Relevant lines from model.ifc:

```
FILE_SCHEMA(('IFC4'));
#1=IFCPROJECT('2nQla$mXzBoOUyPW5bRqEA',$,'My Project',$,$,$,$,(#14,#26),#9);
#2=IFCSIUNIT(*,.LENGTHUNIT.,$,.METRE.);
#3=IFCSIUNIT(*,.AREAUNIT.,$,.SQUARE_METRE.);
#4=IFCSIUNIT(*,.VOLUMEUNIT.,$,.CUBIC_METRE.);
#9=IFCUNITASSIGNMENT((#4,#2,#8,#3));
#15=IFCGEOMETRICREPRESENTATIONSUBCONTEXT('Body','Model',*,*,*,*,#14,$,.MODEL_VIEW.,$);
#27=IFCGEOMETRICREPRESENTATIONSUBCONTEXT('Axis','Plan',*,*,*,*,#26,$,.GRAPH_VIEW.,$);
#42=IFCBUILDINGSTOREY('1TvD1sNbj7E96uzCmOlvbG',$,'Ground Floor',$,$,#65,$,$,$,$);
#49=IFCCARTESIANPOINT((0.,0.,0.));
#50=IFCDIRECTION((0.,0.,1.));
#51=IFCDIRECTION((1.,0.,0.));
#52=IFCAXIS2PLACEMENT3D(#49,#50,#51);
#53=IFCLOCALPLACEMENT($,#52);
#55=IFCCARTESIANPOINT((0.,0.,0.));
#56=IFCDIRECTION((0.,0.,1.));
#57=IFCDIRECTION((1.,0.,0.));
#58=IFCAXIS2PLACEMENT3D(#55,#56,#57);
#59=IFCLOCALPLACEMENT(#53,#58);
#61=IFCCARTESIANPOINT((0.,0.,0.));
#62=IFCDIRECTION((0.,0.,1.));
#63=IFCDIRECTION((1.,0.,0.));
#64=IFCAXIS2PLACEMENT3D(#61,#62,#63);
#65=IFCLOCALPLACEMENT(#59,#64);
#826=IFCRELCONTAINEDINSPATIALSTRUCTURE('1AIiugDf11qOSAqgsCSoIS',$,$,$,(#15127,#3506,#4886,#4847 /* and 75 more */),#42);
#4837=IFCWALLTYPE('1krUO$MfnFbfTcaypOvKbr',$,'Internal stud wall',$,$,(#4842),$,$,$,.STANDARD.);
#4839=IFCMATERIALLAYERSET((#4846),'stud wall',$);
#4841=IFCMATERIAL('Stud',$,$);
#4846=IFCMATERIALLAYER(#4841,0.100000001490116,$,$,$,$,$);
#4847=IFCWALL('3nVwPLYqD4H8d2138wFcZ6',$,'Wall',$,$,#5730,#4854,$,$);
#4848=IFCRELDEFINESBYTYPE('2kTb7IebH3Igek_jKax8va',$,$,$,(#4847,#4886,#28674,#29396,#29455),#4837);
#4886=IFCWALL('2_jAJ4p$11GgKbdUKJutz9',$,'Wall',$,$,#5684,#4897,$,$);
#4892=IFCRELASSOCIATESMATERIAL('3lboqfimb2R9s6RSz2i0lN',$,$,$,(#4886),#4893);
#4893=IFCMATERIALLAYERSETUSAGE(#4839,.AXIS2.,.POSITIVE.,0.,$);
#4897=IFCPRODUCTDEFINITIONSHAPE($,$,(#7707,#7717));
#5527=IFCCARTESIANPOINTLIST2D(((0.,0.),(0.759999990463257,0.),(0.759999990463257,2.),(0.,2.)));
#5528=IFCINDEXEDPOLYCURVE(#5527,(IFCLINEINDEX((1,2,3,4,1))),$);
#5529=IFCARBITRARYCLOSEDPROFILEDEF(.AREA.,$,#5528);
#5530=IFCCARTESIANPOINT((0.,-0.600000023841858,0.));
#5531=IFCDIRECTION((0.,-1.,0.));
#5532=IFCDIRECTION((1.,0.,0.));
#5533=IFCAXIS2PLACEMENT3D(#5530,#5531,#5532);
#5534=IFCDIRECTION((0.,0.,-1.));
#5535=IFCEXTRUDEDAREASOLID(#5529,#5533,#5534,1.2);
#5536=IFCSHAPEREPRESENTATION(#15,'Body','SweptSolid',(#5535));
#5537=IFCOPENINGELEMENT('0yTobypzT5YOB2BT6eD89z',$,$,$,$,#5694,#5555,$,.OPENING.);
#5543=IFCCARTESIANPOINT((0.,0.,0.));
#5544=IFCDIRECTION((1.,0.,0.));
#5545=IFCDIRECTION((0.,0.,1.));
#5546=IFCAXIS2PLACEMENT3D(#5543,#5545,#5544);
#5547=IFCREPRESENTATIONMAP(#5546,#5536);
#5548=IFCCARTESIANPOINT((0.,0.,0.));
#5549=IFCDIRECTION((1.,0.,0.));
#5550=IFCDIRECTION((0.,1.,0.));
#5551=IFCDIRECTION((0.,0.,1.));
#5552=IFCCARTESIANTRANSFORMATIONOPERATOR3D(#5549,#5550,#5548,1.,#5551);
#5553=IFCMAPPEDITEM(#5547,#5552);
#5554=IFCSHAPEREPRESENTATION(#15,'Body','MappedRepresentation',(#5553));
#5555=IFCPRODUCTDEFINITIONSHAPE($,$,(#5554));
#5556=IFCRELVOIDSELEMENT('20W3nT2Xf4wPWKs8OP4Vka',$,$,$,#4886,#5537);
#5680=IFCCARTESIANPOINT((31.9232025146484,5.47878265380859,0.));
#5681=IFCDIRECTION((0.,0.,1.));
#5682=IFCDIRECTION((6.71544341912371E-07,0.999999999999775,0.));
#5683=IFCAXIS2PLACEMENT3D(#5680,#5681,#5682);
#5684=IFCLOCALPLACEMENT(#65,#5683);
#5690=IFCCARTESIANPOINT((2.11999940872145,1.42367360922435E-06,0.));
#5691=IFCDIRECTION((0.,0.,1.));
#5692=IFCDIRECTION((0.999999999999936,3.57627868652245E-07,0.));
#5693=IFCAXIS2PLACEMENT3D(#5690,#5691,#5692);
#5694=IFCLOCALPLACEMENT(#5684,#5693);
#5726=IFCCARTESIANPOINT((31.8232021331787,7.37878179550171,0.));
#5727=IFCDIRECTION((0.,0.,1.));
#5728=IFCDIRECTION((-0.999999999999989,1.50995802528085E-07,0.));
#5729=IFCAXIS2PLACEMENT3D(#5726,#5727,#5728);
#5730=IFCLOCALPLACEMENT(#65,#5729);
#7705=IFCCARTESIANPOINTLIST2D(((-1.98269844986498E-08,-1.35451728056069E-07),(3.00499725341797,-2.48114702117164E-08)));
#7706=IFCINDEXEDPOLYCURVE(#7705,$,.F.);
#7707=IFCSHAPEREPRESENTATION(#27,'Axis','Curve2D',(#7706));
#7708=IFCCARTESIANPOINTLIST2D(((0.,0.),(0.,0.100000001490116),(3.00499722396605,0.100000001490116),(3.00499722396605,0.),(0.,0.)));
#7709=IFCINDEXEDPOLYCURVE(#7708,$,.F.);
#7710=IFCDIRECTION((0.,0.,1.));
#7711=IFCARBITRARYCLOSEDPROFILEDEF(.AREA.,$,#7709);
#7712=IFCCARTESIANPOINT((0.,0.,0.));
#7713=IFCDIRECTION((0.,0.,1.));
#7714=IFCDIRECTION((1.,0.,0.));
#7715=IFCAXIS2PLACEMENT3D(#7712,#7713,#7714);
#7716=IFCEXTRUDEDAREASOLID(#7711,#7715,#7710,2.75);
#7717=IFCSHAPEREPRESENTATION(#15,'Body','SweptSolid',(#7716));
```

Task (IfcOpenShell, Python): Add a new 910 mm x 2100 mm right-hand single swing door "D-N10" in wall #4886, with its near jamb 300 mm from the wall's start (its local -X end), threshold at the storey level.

```python
import numpy as np
import ifcopenshell
import ifcopenshell.api.feature
import ifcopenshell.api.geometry
import ifcopenshell.api.root
import ifcopenshell.api.spatial
import ifcopenshell.geom
import ifcopenshell.util.element
import ifcopenshell.util.placement
import ifcopenshell.util.representation
import ifcopenshell.util.shape
import ifcopenshell.util.unit

model = ifcopenshell.open("model.ifc")
unit_scale = ifcopenshell.util.unit.calculate_unit_scale(model)
settings = ifcopenshell.geom.settings()


def volume(element):
    """Net volume in cubic metres, openings subtracted."""
    shape = ifcopenshell.geom.create_shape(settings, element)
    return ifcopenshell.util.shape.get_volume(shape.geometry)


wall = model.by_id(4886)
storey = ifcopenshell.util.element.get_container(wall, ifc_class="IfcBuildingStorey")
context = ifcopenshell.util.representation.get_context(model, "Model", "Body", "MODEL_VIEW")
before = volume(wall)

width, height, from_end, sill = 0.91, 2.1, 0.3, 0.0  # metres

# The wall runs along its own X axis, and the end named is its -X end.
wall_shape = ifcopenshell.geom.create_shape(settings, wall)
x, y, z = ifcopenshell.util.shape.get_vertices(wall_shape.geometry).T
start = x.min() + from_end
face, thickness = float(y.min()), float(y.max() - y.min())
wall_matrix = ifcopenshell.util.placement.get_local_placement(wall.ObjectPlacement)
level = ifcopenshell.util.placement.get_local_placement(storey.ObjectPlacement)[2, 3]


def in_wall(x, y):
    """Placement at x, y metres in the wall's axes, at sill height."""
    matrix = wall_matrix.copy()
    matrix[:, 3] = wall_matrix @ np.array([x / unit_scale, y / unit_scale, 0.0, 1.0])
    matrix[2, 3] = level + sill / unit_scale
    return matrix


# Opening: a box that overshoots both wall faces by 50 mm.
opening = ifcopenshell.api.root.create_entity(model, ifc_class="IfcOpeningElement", predefined_type="OPENING")
box = ifcopenshell.api.geometry.add_wall_representation(
    model, context=context, length=width, height=height, thickness=thickness + 0.1
)
ifcopenshell.api.geometry.assign_representation(model, product=opening, representation=box)
ifcopenshell.api.geometry.edit_object_placement(model, product=opening, matrix=in_wall(start, face - 0.05), is_si=False)
ifcopenshell.api.feature.add_feature(model, feature=opening, element=wall)

door = ifcopenshell.api.root.create_entity(model, ifc_class="IfcDoor", name="D-N10", predefined_type="DOOR")
door.OverallWidth, door.OverallHeight = width / unit_scale, height / unit_scale
door.OperationType = "SINGLE_SWING_RIGHT"
body = ifcopenshell.api.geometry.add_door_representation(
    model,
    context=context,
    overall_width=door.OverallWidth,
    overall_height=door.OverallHeight,
    operation_type="SINGLE_SWING_RIGHT",
    lining_properties={"LiningDepth": thickness / unit_scale, "ThresholdDepth": thickness / unit_scale},
)
ifcopenshell.api.geometry.assign_representation(model, product=door, representation=body)
ifcopenshell.api.spatial.assign_container(model, products=[door], relating_structure=storey)
ifcopenshell.api.feature.add_filling(model, opening=opening, element=door)

# The lining spans the wall, so the door starts at the wall face.
ifcopenshell.api.geometry.edit_object_placement(model, product=door, matrix=in_wall(start, face), is_si=False)

after = volume(wall)

print(f"wall volume {before:.3f} -> {after:.3f} m3")

model.write("model_updated.ifc")
```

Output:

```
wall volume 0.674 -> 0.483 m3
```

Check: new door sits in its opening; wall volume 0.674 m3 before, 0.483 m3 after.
